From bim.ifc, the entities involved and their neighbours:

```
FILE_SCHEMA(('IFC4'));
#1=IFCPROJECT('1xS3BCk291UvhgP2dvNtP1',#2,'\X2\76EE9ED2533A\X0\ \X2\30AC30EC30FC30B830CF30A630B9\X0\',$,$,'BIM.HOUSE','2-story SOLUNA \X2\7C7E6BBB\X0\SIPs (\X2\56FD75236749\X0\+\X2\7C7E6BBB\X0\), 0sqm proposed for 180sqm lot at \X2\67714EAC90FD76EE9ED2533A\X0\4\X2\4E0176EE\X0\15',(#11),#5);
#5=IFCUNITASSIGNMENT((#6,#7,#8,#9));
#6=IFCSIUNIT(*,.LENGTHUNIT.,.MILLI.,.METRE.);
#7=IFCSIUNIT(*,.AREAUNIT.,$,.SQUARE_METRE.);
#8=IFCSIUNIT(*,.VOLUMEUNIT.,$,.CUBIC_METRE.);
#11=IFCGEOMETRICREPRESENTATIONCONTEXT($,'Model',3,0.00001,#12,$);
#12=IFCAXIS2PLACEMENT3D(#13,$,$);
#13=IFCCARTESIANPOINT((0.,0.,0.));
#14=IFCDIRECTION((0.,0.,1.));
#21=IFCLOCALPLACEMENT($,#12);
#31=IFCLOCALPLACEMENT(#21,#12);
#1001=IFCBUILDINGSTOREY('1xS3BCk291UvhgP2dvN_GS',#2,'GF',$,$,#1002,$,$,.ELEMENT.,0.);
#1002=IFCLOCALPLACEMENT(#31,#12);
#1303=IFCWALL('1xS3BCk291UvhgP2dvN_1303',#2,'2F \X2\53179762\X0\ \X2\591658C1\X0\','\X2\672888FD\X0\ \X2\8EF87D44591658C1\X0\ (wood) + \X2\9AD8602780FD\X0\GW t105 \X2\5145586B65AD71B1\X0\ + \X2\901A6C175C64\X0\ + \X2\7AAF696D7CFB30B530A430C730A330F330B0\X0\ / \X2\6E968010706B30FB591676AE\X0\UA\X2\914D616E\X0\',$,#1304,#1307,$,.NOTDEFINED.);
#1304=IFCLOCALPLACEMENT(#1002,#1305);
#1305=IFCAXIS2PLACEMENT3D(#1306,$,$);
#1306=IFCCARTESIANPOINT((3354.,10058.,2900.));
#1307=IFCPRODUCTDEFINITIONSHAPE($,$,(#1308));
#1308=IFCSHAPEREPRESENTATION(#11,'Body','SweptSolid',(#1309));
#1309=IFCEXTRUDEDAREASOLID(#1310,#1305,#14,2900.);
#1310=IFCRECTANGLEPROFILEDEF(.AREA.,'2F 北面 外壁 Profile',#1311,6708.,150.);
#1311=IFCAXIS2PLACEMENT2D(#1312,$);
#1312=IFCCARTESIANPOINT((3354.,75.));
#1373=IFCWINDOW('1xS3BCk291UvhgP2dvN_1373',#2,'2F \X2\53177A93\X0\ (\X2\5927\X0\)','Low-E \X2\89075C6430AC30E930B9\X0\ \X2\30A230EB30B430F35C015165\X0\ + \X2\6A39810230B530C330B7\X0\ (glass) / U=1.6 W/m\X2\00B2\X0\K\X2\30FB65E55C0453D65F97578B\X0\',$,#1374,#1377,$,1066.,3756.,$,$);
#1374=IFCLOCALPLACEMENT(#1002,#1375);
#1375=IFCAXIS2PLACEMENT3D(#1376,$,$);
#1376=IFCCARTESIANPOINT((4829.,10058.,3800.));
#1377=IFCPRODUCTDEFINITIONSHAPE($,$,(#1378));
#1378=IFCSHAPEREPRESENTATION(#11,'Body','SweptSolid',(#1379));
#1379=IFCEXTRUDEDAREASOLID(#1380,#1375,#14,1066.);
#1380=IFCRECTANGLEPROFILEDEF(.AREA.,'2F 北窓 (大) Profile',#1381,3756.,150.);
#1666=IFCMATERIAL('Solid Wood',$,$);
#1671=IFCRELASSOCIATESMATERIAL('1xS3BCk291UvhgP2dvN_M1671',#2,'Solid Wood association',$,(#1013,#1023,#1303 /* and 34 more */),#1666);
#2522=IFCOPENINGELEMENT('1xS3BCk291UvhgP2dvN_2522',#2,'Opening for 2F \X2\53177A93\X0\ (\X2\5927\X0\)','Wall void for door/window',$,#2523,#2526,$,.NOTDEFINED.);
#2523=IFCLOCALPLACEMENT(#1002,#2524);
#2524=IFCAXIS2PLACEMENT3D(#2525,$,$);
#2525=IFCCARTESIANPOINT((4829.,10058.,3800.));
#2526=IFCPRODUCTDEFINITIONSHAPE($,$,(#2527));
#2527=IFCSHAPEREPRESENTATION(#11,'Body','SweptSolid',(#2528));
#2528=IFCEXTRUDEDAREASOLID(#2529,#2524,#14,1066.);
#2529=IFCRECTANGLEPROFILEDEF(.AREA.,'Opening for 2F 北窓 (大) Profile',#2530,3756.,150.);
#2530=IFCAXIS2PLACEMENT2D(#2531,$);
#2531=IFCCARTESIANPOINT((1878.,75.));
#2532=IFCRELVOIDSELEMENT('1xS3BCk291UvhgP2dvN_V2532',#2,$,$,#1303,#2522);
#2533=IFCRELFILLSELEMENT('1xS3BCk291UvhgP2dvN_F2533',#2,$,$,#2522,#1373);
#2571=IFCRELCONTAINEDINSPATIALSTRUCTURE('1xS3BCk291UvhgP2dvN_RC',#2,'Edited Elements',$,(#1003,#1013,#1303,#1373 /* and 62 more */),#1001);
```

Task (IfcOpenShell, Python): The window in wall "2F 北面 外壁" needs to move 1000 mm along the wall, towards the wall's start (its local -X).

```python
import ifcopenshell
import ifcopenshell.api.geometry
import ifcopenshell.util.placement
import ifcopenshell.util.unit

model = ifcopenshell.open("bim.ifc")
unit_scale = ifcopenshell.util.unit.calculate_unit_scale(model)

window = model.by_id(1373)
opening = window.FillsVoids[0].RelatingOpeningElement
wall = opening.VoidsElements[0].RelatingBuildingElement

wall_matrix = ifcopenshell.util.placement.get_local_placement(wall.ObjectPlacement)
shift = wall_matrix[:3, 0] * -1 / unit_scale
before = ifcopenshell.util.placement.get_local_placement(window.ObjectPlacement)[:3, 3].copy()

# The window is not placed relative to its opening, so move both.
for product in (opening, window):
    matrix = ifcopenshell.util.placement.get_local_placement(product.ObjectPlacement)
    matrix[:3, 3] += shift
    ifcopenshell.api.geometry.edit_object_placement(model, product=product, matrix=matrix, is_si=False)

after = ifcopenshell.util.placement.get_local_placement(window.ObjectPlacement)[:3, 3]
print("window moved by", (after - before).round(3) + 0.0)

model.write("bim_rev.ifc")
```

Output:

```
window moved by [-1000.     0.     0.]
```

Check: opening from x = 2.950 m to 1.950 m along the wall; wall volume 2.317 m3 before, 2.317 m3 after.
